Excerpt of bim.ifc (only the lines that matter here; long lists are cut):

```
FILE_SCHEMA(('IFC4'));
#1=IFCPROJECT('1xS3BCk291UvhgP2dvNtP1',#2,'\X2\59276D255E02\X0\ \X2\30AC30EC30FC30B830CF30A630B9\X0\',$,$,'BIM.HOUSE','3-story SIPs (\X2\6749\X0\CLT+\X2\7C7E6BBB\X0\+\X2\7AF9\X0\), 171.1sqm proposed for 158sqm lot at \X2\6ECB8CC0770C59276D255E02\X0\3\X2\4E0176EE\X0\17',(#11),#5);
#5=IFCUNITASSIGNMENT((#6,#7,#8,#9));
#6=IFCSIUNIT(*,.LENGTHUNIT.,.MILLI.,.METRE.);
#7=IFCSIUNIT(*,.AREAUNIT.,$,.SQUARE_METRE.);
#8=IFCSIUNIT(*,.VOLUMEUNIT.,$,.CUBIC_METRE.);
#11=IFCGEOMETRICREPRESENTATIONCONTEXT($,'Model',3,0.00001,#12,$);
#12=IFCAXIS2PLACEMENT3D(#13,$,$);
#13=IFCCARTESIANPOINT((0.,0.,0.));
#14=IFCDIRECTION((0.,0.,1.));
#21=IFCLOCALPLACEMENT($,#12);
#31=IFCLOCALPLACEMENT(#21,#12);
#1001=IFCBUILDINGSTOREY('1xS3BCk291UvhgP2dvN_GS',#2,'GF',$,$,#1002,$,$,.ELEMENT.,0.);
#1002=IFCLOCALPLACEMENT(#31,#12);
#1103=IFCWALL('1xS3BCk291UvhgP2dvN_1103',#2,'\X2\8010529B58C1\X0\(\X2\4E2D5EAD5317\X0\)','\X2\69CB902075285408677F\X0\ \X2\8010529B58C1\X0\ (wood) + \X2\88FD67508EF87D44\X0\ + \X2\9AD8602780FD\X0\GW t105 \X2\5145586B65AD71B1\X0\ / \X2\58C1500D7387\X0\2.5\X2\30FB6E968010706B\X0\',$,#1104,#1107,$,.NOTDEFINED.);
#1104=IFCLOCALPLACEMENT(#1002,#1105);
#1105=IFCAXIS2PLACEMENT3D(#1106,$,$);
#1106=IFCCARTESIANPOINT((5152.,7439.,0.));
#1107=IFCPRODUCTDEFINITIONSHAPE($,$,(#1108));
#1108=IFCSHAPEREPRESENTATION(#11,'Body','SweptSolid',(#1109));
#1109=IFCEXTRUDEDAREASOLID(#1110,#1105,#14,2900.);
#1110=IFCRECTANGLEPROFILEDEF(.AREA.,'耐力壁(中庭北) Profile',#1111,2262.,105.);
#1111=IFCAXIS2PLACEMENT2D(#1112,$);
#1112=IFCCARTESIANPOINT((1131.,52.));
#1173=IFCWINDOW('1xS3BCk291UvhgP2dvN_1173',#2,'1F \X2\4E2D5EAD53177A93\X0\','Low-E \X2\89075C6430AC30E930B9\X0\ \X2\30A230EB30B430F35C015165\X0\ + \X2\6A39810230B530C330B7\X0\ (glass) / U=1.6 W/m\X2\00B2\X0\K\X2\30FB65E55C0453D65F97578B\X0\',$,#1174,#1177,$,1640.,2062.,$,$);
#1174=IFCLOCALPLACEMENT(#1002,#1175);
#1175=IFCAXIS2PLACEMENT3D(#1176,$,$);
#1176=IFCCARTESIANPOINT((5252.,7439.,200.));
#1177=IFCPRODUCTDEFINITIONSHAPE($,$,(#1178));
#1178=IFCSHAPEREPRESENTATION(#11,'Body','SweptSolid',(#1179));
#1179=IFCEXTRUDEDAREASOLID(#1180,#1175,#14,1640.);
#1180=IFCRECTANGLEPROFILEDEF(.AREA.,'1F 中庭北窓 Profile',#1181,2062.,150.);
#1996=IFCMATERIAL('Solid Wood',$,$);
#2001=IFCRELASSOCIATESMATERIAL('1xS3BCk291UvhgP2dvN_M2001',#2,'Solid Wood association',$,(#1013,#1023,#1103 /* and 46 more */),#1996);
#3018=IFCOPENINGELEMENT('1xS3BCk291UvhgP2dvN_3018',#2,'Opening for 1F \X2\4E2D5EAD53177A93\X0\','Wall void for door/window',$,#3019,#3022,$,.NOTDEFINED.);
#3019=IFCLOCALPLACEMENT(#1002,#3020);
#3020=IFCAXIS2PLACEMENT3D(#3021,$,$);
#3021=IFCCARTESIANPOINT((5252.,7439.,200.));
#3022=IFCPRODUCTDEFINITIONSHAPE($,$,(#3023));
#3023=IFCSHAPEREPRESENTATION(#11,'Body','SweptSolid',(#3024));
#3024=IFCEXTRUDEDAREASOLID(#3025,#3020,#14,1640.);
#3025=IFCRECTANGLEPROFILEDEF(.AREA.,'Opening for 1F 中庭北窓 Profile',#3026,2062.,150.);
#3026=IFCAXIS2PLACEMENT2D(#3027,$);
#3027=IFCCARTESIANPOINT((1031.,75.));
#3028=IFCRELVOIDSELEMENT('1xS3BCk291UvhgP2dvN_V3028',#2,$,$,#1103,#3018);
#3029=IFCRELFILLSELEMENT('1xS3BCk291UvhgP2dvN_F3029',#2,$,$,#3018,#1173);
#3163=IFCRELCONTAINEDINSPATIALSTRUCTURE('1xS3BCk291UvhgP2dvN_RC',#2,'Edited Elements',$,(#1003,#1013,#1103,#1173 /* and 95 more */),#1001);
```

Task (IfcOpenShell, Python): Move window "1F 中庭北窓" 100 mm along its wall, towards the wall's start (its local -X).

```python
import ifcopenshell
import ifcopenshell.api.geometry
import ifcopenshell.util.placement
import ifcopenshell.util.unit

model = ifcopenshell.open("bim.ifc")
unit_scale = ifcopenshell.util.unit.calculate_unit_scale(model)

window = model.by_guid("1xS3BCk291UvhgP2dvN_1173")
opening = window.FillsVoids[0].RelatingOpeningElement
wall = opening.VoidsElements[0].RelatingBuildingElement

wall_matrix = ifcopenshell.util.placement.get_local_placement(wall.ObjectPlacement)
shift = wall_matrix[:3, 0] * -0.1 / unit_scale
before = ifcopenshell.util.placement.get_local_placement(window.ObjectPlacement)[:3, 3].copy()

# The window is not placed relative to its opening, so move both.
for product in (opening, window):
    matrix = ifcopenshell.util.placement.get_local_placement(product.ObjectPlacement)
    matrix[:3, 3] += shift
    ifcopenshell.api.geometry.edit_object_placement(model, product=product, matrix=matrix, is_si=False)

after = ifcopenshell.util.placement.get_local_placement(window.ObjectPlacement)[:3, 3]
print("window moved by", (after - before).round(3) + 0.0)

model.write("bim_v2.ifc")
```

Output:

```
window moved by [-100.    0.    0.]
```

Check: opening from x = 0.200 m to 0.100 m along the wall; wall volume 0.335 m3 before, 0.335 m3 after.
